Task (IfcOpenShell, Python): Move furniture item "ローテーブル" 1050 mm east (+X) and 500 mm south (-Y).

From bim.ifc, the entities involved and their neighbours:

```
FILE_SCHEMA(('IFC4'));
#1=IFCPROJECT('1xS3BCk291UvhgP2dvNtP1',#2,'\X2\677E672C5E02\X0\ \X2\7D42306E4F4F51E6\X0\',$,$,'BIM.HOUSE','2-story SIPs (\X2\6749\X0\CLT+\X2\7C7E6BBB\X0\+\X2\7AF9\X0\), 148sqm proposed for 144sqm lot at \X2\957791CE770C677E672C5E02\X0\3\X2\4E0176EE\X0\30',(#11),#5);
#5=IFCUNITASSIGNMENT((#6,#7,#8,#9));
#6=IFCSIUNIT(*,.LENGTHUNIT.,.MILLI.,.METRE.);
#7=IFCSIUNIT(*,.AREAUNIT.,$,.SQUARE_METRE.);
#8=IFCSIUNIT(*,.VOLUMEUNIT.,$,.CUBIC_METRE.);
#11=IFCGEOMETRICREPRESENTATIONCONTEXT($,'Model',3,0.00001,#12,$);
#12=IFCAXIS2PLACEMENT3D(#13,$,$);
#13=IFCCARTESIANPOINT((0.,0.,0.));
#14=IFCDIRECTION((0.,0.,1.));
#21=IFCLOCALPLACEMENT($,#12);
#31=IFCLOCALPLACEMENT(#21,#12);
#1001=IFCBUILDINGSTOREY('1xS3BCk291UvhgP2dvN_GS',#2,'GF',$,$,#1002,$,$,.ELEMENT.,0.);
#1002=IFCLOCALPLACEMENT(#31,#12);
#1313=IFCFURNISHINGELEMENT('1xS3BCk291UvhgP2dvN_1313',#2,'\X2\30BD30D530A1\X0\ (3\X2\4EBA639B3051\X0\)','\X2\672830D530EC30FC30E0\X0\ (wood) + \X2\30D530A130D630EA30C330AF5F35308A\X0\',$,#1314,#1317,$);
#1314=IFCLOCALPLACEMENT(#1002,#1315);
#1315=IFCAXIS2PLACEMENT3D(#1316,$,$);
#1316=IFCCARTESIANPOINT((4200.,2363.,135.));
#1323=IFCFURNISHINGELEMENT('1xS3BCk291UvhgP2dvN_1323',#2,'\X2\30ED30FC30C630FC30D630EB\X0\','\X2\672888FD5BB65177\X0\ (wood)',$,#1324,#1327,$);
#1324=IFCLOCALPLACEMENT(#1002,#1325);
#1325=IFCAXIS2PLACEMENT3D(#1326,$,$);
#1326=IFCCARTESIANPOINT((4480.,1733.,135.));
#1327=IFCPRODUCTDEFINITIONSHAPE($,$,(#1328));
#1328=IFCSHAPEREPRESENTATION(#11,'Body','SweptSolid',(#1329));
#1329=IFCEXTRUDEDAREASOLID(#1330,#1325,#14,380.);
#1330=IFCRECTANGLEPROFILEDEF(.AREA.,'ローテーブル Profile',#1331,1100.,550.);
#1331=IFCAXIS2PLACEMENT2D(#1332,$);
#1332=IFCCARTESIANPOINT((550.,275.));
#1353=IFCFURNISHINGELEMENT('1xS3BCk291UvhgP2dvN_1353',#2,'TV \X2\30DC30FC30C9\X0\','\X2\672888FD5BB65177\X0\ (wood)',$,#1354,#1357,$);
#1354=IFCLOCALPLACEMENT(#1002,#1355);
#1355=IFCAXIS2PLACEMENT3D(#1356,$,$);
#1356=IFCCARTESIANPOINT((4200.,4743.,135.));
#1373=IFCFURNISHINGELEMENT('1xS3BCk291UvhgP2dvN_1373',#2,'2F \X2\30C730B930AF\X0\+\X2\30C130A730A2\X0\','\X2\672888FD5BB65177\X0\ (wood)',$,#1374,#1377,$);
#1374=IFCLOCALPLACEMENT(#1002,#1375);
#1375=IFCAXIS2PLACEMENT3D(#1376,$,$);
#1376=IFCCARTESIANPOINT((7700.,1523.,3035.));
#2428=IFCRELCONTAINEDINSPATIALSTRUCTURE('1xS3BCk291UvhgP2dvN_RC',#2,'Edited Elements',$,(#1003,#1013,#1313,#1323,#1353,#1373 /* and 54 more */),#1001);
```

```python
import ifcopenshell
import ifcopenshell.api.geometry
import ifcopenshell.util.placement
import ifcopenshell.util.unit

model = ifcopenshell.open("bim.ifc")
unit_scale = ifcopenshell.util.unit.calculate_unit_scale(model)

item = model.by_guid("1xS3BCk291UvhgP2dvN_1323")
matrix = ifcopenshell.util.placement.get_local_placement(item.ObjectPlacement)
matrix[0, 3] += 1.05 / unit_scale
matrix[1, 3] -= 0.5 / unit_scale
ifcopenshell.api.geometry.edit_object_placement(model, product=item, matrix=matrix, is_si=False)

print(ifcopenshell.util.placement.get_local_placement(item.ObjectPlacement).round(3) + 0.0)

model.write("bim_updated.ifc")
```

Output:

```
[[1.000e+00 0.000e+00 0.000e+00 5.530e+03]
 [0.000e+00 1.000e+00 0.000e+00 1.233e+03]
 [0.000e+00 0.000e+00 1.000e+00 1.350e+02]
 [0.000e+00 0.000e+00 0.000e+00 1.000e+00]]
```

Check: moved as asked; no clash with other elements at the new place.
